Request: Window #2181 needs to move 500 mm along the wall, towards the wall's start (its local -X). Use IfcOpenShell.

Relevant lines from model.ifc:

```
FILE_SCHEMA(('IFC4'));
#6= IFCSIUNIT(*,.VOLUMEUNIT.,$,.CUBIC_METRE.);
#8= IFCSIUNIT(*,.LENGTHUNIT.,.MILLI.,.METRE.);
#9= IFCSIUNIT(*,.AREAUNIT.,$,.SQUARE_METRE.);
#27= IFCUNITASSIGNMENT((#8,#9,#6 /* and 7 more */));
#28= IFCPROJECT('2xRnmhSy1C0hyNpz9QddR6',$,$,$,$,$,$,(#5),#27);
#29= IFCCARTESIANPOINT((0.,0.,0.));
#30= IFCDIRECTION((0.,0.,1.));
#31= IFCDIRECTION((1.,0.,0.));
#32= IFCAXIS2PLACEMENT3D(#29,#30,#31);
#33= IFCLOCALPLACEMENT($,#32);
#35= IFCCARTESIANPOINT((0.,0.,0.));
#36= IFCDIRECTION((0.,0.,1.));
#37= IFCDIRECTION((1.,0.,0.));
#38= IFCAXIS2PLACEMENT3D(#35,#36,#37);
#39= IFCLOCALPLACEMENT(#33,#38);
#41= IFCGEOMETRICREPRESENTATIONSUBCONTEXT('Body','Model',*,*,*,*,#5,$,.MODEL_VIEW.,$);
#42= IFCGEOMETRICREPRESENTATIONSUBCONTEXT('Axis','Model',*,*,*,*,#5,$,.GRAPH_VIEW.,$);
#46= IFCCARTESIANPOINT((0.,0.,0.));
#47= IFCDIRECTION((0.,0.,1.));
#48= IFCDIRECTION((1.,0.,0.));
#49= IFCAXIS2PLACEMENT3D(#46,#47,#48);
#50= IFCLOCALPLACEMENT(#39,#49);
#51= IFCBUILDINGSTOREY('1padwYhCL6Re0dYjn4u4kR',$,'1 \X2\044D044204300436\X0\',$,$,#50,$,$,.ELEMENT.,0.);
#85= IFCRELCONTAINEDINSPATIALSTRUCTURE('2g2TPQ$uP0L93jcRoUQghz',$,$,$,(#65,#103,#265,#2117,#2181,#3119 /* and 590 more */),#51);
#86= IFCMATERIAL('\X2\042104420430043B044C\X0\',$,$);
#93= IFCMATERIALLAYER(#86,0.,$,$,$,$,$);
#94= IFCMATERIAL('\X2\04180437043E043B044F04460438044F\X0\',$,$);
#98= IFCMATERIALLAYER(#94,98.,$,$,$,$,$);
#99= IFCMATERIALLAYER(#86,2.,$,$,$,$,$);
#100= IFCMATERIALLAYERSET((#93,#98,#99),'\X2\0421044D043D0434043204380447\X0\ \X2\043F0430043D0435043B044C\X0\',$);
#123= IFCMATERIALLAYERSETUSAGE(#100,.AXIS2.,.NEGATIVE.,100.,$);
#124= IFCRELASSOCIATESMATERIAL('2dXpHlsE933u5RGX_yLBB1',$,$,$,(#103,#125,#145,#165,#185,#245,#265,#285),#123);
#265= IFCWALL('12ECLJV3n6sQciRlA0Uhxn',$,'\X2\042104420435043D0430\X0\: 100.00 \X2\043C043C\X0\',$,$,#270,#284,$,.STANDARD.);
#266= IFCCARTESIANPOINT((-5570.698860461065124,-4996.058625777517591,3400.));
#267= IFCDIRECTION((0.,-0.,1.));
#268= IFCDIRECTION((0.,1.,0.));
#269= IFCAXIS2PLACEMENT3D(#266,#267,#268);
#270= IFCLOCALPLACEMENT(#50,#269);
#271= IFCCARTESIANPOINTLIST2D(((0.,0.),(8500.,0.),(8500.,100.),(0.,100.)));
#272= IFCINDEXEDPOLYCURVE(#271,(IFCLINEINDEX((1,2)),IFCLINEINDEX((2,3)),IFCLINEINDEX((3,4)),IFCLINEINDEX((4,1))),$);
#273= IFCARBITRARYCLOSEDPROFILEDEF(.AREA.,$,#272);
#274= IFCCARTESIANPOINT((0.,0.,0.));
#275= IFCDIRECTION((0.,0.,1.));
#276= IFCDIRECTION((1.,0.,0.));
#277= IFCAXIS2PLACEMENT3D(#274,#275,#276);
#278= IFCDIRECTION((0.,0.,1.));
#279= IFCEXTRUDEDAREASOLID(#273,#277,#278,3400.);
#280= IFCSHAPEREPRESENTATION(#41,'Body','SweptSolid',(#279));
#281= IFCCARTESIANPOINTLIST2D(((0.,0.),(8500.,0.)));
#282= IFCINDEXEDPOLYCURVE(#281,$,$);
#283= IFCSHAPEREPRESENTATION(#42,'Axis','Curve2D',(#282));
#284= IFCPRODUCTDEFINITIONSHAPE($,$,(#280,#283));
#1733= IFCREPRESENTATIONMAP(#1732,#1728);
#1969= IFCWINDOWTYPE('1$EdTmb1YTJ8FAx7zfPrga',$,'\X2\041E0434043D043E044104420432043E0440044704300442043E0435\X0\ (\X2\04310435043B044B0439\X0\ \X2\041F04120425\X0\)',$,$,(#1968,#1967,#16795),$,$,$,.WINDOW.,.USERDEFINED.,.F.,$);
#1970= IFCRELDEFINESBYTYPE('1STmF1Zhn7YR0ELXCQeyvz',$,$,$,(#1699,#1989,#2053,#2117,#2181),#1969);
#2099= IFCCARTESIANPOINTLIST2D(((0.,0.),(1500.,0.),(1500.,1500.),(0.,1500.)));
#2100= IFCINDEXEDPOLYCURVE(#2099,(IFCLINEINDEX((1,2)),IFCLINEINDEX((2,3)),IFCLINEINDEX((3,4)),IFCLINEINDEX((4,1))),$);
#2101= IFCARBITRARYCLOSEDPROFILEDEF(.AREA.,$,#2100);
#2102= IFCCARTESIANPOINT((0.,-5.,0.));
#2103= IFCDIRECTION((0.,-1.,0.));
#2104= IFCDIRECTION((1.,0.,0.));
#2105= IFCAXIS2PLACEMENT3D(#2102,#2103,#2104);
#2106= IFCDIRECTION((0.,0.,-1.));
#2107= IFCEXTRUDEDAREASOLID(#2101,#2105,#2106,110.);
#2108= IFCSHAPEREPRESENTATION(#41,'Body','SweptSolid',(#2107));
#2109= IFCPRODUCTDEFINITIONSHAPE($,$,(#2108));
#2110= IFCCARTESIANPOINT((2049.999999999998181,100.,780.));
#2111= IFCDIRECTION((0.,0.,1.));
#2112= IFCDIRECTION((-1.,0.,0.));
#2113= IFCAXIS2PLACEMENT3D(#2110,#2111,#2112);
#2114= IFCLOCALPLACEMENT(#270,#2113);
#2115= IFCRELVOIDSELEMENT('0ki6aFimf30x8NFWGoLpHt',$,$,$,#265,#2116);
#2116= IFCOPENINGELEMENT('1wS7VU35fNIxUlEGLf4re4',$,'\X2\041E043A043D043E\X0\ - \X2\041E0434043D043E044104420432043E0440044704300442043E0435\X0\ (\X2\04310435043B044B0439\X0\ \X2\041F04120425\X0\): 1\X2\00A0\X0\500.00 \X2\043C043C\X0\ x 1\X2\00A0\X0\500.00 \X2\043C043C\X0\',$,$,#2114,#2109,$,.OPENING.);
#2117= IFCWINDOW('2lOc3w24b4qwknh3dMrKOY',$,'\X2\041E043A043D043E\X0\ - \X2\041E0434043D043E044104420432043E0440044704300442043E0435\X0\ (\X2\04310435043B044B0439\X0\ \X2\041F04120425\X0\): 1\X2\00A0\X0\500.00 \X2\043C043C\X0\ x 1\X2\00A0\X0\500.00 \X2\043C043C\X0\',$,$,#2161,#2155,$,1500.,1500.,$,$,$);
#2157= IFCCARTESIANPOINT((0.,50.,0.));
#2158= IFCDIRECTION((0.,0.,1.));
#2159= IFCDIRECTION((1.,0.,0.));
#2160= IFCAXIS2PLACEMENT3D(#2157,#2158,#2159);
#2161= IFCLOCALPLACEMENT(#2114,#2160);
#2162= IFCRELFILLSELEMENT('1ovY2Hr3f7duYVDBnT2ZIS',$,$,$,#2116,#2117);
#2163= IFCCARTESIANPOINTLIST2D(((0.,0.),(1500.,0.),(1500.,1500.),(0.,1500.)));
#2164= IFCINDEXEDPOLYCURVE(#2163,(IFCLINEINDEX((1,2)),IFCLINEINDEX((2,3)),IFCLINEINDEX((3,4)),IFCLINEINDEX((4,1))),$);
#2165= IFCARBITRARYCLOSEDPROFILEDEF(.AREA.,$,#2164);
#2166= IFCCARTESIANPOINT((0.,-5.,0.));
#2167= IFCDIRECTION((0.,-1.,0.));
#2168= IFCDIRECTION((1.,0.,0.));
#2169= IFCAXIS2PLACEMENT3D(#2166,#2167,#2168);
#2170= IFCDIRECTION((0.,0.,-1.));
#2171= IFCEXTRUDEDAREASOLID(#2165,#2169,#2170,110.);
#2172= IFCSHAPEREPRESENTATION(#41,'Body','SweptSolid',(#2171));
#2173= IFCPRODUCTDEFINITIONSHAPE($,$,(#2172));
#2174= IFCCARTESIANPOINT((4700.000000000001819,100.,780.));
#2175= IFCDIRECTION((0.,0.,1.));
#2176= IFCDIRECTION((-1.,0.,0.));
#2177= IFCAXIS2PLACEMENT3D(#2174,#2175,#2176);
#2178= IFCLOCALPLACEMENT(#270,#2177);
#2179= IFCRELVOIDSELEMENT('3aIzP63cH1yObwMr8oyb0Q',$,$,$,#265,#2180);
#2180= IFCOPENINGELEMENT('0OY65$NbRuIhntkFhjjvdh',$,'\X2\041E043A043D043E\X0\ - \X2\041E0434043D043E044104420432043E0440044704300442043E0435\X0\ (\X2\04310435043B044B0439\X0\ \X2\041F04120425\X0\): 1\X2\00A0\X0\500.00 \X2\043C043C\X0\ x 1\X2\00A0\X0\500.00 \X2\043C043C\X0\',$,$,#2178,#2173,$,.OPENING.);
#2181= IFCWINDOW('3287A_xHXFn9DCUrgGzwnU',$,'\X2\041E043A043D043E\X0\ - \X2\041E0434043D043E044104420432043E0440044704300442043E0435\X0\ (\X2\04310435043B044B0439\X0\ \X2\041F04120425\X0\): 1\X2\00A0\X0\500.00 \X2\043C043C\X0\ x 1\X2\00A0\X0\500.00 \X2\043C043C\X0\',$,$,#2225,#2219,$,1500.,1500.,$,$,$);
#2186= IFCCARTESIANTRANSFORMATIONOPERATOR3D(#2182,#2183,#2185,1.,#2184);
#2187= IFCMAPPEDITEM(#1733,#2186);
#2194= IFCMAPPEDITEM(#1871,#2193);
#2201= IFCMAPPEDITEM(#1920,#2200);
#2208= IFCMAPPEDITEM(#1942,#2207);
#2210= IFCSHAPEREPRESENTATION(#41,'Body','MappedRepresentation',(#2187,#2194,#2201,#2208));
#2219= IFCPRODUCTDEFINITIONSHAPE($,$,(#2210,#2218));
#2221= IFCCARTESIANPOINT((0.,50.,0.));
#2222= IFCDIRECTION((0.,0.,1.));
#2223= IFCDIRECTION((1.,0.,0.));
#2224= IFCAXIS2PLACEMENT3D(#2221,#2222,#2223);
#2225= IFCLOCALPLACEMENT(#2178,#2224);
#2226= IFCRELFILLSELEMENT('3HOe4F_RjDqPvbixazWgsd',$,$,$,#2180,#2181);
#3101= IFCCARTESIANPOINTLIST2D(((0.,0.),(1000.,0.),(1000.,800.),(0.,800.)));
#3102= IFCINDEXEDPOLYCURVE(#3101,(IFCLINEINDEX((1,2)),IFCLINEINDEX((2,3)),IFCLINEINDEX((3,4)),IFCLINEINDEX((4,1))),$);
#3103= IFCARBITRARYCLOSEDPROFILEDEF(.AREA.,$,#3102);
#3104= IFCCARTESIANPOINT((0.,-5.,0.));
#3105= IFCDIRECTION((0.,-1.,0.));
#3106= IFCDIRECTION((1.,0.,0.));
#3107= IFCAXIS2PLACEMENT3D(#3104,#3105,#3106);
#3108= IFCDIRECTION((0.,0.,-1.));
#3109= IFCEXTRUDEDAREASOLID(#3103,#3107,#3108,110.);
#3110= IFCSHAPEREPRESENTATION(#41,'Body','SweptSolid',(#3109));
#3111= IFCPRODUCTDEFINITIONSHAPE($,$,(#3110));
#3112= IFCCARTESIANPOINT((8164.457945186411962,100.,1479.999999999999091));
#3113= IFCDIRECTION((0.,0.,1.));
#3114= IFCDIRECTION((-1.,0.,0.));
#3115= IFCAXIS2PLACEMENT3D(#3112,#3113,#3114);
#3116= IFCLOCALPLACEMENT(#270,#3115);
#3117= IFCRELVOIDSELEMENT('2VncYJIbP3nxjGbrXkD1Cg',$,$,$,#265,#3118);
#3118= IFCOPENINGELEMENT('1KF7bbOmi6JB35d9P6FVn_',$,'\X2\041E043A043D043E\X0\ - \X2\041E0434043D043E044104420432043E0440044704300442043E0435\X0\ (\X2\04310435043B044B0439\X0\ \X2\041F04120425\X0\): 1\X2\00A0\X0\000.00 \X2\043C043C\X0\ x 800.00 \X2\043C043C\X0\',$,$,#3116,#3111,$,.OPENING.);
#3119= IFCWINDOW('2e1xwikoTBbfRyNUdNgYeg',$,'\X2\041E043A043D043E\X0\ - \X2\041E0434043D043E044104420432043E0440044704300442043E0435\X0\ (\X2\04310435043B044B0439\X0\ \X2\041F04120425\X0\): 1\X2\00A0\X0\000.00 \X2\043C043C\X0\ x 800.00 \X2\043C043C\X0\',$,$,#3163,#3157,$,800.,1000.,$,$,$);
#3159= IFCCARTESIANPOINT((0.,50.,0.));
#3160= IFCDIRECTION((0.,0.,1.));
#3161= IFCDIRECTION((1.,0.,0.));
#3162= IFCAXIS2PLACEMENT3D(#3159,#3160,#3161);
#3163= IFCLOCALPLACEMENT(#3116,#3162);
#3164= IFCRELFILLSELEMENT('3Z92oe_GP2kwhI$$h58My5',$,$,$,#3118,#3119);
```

```python
import ifcopenshell
import ifcopenshell.api.geometry
import ifcopenshell.util.placement

model = ifcopenshell.open("model.ifc")

window = model.by_id(2181)
opening = window.FillsVoids[0].RelatingOpeningElement
wall = opening.VoidsElements[0].RelatingBuildingElement

wall_matrix = ifcopenshell.util.placement.get_local_placement(wall.ObjectPlacement)
shift = wall_matrix[:3, 0] * -500.0
before = ifcopenshell.util.placement.get_local_placement(window.ObjectPlacement)[:3, 3].copy()

# The window is placed relative to its opening, so it follows when the opening moves.
matrix = ifcopenshell.util.placement.get_local_placement(opening.ObjectPlacement)
matrix[:3, 3] += shift
ifcopenshell.api.geometry.edit_object_placement(
    model, product=opening, matrix=matrix, is_si=False, should_transform_children=True
)

after = ifcopenshell.util.placement.get_local_placement(window.ObjectPlacement)[:3, 3]
print("window moved by", (after - before).round(3) + 0.0)

model.write("model_updated.ifc")
```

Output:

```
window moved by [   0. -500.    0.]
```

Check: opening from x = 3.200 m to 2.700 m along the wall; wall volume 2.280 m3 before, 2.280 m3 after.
